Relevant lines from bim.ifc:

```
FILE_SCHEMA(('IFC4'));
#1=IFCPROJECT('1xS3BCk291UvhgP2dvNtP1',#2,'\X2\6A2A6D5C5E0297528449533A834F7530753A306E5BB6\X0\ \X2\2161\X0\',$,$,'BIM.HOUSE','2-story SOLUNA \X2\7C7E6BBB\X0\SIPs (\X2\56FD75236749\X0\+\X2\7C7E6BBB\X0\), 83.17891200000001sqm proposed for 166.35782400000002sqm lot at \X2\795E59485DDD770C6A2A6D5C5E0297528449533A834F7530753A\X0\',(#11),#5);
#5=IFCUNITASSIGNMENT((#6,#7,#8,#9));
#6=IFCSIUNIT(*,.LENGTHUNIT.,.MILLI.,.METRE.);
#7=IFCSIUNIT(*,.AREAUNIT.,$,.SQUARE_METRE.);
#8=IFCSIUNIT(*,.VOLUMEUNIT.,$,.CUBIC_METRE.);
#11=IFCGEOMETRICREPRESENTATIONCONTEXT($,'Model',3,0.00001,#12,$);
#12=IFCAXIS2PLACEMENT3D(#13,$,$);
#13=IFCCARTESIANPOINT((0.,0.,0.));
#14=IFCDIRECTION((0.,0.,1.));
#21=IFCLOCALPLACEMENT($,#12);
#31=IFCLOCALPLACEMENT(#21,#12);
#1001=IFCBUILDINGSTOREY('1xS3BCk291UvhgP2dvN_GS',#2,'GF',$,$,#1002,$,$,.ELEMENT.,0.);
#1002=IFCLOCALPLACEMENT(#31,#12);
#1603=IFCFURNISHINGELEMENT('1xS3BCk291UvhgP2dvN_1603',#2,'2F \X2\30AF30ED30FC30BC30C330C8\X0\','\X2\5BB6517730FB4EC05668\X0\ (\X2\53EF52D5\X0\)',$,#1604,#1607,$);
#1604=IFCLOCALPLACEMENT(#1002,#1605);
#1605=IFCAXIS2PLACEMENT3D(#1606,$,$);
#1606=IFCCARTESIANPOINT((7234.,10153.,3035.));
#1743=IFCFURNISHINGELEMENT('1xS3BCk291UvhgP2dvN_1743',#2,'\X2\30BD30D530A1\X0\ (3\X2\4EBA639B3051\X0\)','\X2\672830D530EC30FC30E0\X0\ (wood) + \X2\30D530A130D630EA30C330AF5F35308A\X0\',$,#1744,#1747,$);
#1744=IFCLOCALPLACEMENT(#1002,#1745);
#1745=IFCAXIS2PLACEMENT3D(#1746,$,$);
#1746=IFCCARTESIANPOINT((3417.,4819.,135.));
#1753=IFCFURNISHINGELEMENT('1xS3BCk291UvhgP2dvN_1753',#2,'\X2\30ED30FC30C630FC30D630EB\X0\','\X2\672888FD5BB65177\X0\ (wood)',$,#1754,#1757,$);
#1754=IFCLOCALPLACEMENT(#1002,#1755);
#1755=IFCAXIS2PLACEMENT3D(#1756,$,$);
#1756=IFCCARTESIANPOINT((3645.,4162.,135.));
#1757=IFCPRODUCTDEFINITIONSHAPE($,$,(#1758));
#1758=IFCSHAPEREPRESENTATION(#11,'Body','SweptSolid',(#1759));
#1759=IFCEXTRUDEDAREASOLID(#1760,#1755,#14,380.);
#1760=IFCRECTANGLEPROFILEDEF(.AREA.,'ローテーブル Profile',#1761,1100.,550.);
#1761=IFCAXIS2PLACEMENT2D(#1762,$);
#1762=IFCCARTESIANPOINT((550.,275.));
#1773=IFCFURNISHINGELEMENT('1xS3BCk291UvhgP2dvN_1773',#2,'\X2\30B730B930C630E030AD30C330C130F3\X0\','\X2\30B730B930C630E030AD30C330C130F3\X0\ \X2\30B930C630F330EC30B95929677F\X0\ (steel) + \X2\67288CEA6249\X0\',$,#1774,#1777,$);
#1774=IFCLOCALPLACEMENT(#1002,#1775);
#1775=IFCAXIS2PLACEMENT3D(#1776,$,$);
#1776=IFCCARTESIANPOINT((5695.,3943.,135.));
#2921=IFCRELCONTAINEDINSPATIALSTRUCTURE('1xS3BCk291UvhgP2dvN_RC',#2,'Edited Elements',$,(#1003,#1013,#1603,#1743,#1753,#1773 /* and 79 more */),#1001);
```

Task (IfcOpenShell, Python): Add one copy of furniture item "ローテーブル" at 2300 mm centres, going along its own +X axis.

```python
import ifcopenshell
import ifcopenshell.api.geometry
import ifcopenshell.api.root
import ifcopenshell.util.element
import ifcopenshell.util.placement
import ifcopenshell.util.unit

model = ifcopenshell.open("bim.ifc")
unit_scale = ifcopenshell.util.unit.calculate_unit_scale(model)


def reuse_history(source, copy):
    """copy_class also copies each property set's owner history, people and application; keep the originals."""
    for rel in copy.IsDefinedBy:
        if rel.is_a("IfcRelDefinesByProperties") and (history := rel.RelatingPropertyDefinition.OwnerHistory):
            rel.RelatingPropertyDefinition.OwnerHistory = source.OwnerHistory
            ifcopenshell.util.element.remove_deep2(model, history)


source = model.by_guid("1xS3BCk291UvhgP2dvN_1753")
base = ifcopenshell.util.placement.get_local_placement(source.ObjectPlacement)
step = base[:3, 0] * 2.3 / unit_scale

for i in range(1, 2):
    copy = ifcopenshell.api.root.copy_class(model, product=source)
    copy.Representation = ifcopenshell.util.element.copy_deep(
        model, source.Representation, exclude=["IfcGeometricRepresentationContext", "IfcRepresentationMap"]
    )
    reuse_history(source, copy)
    matrix = base.copy()
    matrix[:3, 3] += i * step
    print("added at", matrix[:3, 3].round(3) + 0.0)
    ifcopenshell.api.geometry.edit_object_placement(model, product=copy, matrix=matrix, is_si=False)

model.write("bim-out.ifc")
```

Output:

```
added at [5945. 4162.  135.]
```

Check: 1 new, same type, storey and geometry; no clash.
